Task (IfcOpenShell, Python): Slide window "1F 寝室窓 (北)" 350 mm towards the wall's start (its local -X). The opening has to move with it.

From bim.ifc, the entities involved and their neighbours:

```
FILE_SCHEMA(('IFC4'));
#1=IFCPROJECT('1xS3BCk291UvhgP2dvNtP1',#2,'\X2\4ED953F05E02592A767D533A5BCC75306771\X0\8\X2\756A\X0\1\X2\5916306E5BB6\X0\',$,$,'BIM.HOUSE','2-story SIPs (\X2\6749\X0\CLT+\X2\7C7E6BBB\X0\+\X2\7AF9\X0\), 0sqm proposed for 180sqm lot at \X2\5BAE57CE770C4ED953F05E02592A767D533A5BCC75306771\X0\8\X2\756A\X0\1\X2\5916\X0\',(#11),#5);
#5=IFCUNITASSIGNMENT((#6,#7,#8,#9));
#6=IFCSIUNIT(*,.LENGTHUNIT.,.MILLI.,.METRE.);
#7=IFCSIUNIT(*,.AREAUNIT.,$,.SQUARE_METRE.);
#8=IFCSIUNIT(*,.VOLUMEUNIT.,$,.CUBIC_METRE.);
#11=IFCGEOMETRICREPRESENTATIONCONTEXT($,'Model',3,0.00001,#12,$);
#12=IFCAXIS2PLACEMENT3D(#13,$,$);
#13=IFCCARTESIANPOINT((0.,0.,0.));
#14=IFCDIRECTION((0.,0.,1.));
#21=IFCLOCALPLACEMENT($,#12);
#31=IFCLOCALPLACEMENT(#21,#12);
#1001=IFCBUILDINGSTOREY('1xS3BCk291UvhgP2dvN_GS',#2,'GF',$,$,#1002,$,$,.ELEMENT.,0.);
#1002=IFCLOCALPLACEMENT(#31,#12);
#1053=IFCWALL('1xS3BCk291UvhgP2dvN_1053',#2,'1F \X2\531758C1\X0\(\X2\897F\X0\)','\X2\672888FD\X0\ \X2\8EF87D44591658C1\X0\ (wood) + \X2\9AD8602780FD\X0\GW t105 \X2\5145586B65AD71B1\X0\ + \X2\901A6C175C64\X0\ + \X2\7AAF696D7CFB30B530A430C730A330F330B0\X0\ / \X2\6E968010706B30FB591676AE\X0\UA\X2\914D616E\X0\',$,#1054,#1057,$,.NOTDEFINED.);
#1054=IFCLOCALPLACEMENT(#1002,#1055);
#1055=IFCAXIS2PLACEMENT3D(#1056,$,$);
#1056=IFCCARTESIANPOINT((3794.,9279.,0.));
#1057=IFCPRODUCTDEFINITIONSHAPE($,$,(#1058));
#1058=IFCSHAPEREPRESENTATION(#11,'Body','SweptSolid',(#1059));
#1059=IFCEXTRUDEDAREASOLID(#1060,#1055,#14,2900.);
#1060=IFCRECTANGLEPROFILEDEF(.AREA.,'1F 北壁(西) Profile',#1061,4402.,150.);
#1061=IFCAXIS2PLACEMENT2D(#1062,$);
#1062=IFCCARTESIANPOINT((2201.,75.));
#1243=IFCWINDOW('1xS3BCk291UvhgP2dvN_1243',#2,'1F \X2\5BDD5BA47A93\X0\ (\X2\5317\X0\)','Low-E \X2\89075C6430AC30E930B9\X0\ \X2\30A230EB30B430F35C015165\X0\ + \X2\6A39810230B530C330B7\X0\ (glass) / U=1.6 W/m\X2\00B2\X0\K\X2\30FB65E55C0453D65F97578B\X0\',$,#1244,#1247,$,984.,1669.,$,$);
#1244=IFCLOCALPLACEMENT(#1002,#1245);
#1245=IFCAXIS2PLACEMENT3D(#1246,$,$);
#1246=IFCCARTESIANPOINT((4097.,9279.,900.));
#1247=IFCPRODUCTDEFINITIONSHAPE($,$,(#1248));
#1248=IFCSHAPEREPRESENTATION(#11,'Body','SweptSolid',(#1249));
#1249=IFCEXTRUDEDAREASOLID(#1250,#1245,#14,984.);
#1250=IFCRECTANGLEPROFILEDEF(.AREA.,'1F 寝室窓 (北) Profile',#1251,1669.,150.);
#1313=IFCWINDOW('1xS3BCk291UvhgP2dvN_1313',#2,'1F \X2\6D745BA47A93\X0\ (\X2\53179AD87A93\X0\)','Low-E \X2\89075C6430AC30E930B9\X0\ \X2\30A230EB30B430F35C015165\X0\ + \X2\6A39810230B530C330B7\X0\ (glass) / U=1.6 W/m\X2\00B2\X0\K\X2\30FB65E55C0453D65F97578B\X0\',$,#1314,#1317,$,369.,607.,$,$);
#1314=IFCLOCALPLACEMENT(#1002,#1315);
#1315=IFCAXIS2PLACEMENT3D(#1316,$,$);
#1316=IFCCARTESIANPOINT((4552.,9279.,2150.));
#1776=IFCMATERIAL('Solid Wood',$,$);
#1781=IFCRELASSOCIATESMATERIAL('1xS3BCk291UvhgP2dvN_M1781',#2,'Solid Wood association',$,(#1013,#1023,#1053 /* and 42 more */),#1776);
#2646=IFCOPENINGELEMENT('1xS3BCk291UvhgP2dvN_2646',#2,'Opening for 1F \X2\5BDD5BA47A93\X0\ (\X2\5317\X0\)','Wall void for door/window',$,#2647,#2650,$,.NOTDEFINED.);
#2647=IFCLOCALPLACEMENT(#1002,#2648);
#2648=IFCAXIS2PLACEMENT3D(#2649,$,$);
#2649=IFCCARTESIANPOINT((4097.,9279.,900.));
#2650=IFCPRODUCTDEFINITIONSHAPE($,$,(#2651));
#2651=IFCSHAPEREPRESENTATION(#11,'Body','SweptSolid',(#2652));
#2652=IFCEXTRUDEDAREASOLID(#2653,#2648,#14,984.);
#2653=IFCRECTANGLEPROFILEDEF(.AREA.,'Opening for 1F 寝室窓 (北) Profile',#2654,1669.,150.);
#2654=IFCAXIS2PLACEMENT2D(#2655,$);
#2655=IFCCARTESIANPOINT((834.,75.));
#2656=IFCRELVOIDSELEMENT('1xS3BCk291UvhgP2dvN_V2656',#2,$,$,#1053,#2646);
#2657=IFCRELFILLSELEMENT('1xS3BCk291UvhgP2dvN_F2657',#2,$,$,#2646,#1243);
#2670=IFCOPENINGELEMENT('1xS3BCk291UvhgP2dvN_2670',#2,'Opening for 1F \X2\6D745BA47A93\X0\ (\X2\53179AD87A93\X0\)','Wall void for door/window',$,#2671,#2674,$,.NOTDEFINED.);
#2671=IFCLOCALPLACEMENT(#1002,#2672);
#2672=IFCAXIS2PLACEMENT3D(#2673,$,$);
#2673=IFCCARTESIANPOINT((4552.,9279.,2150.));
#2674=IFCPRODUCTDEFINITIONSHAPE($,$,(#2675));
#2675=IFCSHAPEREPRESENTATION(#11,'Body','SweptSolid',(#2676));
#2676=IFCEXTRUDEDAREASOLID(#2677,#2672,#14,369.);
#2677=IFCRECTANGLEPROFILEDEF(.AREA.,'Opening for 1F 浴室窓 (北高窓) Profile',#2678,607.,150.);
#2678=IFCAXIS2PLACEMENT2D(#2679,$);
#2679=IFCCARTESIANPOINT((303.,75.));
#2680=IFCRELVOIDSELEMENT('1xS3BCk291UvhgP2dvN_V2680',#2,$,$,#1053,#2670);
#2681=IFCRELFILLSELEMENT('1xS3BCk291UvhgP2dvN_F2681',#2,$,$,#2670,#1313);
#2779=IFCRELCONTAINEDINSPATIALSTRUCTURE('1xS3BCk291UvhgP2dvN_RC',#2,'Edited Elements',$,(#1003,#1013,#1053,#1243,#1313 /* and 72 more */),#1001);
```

```python
import ifcopenshell
import ifcopenshell.api.geometry
import ifcopenshell.util.placement

model = ifcopenshell.open("bim.ifc")

window = model.by_guid("1xS3BCk291UvhgP2dvN_1243")
opening = window.FillsVoids[0].RelatingOpeningElement
wall = opening.VoidsElements[0].RelatingBuildingElement

wall_matrix = ifcopenshell.util.placement.get_local_placement(wall.ObjectPlacement)
shift = wall_matrix[:3, 0] * -350.0
before = ifcopenshell.util.placement.get_local_placement(window.ObjectPlacement)[:3, 3].copy()

# The window is not placed relative to its opening, so move both.
for product in (opening, window):
    matrix = ifcopenshell.util.placement.get_local_placement(product.ObjectPlacement)
    matrix[:3, 3] += shift
    ifcopenshell.api.geometry.edit_object_placement(model, product=product, matrix=matrix, is_si=False)

after = ifcopenshell.util.placement.get_local_placement(window.ObjectPlacement)[:3, 3]
print("window moved by", (after - before).round(3) + 0.0)

model.write("bim_updated.ifc")
```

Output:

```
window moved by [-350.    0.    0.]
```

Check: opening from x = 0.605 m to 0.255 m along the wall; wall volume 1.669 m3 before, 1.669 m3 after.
